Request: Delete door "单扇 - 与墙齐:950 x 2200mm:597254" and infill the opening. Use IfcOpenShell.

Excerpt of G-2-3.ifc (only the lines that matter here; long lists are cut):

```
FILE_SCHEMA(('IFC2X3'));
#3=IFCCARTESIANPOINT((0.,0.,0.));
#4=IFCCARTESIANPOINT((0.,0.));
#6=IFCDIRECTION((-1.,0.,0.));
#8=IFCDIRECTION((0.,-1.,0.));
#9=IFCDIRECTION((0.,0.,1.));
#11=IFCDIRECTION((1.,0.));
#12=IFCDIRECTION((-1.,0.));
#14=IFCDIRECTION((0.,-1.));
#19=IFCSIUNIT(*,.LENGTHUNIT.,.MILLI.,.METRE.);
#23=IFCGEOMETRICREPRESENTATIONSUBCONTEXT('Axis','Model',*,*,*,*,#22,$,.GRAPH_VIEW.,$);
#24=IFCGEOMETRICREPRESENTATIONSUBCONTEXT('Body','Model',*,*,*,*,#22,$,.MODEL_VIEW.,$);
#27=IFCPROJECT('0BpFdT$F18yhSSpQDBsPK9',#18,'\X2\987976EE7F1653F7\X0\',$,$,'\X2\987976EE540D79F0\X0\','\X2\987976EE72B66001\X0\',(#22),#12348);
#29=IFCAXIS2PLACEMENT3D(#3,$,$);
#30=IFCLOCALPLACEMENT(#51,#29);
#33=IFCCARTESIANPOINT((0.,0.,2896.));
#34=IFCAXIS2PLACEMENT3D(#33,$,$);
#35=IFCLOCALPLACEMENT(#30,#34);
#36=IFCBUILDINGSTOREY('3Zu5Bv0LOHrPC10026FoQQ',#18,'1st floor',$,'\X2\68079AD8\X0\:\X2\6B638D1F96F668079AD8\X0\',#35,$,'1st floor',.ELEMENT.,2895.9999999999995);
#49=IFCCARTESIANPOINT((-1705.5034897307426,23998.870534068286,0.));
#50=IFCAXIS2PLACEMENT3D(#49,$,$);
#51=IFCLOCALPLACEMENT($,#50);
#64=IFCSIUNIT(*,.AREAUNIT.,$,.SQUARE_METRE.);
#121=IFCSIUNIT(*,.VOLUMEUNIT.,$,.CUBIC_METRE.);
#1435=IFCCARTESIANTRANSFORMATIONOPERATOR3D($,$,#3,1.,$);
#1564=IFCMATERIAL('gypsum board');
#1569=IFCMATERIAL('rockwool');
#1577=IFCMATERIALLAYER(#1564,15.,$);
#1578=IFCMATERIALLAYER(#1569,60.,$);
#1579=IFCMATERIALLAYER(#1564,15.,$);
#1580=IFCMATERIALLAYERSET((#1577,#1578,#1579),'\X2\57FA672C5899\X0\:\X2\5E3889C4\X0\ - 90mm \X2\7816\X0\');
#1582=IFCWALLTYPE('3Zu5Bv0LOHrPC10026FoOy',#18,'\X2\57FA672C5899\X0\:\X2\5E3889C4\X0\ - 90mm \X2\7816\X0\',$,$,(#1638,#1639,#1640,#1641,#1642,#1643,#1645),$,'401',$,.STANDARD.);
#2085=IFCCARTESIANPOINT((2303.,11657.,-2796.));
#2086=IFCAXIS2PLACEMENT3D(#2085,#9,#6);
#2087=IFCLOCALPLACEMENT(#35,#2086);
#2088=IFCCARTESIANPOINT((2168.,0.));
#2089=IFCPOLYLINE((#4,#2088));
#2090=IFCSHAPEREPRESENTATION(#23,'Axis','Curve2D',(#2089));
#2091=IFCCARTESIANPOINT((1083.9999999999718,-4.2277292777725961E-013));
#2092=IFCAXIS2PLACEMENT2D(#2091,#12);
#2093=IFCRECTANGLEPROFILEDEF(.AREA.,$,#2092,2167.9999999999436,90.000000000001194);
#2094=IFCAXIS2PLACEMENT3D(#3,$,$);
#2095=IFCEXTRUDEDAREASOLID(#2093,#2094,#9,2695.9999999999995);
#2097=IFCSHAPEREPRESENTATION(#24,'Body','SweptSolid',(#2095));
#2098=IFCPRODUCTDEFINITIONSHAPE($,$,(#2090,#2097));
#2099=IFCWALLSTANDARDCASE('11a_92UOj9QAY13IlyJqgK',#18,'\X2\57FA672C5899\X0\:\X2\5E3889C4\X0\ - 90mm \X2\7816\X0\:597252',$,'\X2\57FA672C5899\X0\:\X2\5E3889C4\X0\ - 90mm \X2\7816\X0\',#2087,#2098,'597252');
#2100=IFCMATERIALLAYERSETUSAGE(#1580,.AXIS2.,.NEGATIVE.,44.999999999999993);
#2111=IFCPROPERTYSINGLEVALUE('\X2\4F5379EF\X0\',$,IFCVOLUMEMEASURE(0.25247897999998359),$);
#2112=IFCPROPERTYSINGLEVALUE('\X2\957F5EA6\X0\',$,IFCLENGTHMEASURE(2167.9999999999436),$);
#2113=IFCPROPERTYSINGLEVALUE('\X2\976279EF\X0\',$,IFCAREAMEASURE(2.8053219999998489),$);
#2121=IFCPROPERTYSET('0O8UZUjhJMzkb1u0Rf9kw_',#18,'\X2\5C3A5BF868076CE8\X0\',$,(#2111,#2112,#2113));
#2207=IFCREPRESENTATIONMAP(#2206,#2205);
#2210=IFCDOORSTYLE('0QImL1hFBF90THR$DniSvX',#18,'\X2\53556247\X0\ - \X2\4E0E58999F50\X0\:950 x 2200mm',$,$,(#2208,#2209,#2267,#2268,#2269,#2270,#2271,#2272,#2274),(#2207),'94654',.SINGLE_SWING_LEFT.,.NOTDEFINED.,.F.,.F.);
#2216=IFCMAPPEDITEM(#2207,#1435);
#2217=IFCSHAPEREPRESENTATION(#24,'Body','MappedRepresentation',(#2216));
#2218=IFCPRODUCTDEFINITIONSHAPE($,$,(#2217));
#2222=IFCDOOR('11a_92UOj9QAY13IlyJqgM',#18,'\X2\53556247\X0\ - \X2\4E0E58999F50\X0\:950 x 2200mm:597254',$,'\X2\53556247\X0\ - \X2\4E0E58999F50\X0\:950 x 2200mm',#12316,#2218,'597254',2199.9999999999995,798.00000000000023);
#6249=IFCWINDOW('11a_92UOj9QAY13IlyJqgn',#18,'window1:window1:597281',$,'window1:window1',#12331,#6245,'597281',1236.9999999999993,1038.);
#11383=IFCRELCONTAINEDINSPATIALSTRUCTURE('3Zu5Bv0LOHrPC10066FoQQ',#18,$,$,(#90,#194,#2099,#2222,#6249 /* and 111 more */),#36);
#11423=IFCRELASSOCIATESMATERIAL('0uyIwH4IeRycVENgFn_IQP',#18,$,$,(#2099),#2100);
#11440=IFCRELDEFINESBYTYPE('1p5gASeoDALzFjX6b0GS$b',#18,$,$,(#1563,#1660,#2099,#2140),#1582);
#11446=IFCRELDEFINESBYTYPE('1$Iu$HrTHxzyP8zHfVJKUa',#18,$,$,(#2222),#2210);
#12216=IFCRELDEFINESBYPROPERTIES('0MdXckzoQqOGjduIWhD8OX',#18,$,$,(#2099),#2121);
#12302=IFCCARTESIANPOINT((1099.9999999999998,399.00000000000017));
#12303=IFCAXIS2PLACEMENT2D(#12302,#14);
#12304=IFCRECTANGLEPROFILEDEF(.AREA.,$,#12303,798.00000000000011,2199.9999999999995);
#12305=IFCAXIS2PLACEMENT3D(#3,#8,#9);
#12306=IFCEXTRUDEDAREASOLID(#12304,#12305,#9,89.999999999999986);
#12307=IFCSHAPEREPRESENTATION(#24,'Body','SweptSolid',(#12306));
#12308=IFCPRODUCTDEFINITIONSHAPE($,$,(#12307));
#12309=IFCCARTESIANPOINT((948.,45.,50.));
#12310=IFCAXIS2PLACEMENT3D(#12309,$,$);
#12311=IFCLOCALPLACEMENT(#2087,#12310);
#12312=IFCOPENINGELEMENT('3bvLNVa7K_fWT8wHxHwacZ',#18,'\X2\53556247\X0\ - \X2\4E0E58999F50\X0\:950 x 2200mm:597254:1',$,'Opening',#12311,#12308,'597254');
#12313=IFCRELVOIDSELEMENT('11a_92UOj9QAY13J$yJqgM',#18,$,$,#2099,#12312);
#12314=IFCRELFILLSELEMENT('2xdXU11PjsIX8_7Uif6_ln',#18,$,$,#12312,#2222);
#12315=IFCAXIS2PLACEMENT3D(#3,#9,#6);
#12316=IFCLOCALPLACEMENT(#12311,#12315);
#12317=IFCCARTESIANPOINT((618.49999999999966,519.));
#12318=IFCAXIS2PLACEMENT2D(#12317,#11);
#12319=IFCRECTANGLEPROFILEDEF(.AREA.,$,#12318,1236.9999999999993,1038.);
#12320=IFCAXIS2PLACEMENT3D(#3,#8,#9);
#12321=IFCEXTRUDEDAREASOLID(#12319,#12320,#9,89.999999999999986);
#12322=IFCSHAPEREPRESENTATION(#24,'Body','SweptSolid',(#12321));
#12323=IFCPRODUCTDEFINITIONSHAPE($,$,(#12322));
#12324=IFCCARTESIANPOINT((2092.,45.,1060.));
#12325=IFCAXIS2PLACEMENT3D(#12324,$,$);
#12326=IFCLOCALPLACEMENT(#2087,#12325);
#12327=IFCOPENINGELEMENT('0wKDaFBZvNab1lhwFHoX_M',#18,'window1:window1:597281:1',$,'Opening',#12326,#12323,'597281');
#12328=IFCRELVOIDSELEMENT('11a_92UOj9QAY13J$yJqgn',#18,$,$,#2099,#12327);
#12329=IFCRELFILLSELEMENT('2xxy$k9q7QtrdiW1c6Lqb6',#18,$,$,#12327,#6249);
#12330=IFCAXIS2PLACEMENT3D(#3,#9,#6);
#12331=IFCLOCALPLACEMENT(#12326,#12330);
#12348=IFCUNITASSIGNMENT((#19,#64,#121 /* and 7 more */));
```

```python
import ifcopenshell
import ifcopenshell.api.feature
import ifcopenshell.api.pset
import ifcopenshell.api.root
import ifcopenshell.geom
import ifcopenshell.util.element
import ifcopenshell.util.shape
import ifcopenshell.util.unit

model = ifcopenshell.open("G-2-3.ifc")
area_scale = ifcopenshell.util.unit.calculate_unit_scale(model, "AREAUNIT")
volume_scale = ifcopenshell.util.unit.calculate_unit_scale(model, "VOLUMEUNIT")
settings = ifcopenshell.geom.settings()


def volume(element):
    """Net volume in cubic metres, openings subtracted."""
    shape = ifcopenshell.geom.create_shape(settings, element)
    return ifcopenshell.util.shape.get_volume(shape.geometry)


door = model.by_guid("11a_92UOj9QAY13IlyJqgM")
opening = door.FillsVoids[0].RelatingOpeningElement
wall = opening.VoidsElements[0].RelatingBuildingElement
before = volume(wall)

ifcopenshell.api.root.remove_product(model, product=door)
ifcopenshell.api.feature.remove_feature(model, feature=opening)

after = volume(wall)
thickness = 0.09  # wall thickness in metres

# Update the wall's stored quantities.
pset = model.by_id(ifcopenshell.util.element.get_pset(wall, "尺寸标注", should_inherit=False)["id"])
ifcopenshell.api.pset.edit_pset(model, pset=pset, properties={
    "体积": model.create_entity("IfcVolumeMeasure", after / volume_scale),
    "面积": model.create_entity("IfcAreaMeasure", after / thickness / area_scale),
})

print(f"wall volume {before:.3f} -> {after:.3f} m3")

model.write("G-2-3-out.ifc")
```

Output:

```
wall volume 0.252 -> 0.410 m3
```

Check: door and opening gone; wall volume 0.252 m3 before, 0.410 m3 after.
